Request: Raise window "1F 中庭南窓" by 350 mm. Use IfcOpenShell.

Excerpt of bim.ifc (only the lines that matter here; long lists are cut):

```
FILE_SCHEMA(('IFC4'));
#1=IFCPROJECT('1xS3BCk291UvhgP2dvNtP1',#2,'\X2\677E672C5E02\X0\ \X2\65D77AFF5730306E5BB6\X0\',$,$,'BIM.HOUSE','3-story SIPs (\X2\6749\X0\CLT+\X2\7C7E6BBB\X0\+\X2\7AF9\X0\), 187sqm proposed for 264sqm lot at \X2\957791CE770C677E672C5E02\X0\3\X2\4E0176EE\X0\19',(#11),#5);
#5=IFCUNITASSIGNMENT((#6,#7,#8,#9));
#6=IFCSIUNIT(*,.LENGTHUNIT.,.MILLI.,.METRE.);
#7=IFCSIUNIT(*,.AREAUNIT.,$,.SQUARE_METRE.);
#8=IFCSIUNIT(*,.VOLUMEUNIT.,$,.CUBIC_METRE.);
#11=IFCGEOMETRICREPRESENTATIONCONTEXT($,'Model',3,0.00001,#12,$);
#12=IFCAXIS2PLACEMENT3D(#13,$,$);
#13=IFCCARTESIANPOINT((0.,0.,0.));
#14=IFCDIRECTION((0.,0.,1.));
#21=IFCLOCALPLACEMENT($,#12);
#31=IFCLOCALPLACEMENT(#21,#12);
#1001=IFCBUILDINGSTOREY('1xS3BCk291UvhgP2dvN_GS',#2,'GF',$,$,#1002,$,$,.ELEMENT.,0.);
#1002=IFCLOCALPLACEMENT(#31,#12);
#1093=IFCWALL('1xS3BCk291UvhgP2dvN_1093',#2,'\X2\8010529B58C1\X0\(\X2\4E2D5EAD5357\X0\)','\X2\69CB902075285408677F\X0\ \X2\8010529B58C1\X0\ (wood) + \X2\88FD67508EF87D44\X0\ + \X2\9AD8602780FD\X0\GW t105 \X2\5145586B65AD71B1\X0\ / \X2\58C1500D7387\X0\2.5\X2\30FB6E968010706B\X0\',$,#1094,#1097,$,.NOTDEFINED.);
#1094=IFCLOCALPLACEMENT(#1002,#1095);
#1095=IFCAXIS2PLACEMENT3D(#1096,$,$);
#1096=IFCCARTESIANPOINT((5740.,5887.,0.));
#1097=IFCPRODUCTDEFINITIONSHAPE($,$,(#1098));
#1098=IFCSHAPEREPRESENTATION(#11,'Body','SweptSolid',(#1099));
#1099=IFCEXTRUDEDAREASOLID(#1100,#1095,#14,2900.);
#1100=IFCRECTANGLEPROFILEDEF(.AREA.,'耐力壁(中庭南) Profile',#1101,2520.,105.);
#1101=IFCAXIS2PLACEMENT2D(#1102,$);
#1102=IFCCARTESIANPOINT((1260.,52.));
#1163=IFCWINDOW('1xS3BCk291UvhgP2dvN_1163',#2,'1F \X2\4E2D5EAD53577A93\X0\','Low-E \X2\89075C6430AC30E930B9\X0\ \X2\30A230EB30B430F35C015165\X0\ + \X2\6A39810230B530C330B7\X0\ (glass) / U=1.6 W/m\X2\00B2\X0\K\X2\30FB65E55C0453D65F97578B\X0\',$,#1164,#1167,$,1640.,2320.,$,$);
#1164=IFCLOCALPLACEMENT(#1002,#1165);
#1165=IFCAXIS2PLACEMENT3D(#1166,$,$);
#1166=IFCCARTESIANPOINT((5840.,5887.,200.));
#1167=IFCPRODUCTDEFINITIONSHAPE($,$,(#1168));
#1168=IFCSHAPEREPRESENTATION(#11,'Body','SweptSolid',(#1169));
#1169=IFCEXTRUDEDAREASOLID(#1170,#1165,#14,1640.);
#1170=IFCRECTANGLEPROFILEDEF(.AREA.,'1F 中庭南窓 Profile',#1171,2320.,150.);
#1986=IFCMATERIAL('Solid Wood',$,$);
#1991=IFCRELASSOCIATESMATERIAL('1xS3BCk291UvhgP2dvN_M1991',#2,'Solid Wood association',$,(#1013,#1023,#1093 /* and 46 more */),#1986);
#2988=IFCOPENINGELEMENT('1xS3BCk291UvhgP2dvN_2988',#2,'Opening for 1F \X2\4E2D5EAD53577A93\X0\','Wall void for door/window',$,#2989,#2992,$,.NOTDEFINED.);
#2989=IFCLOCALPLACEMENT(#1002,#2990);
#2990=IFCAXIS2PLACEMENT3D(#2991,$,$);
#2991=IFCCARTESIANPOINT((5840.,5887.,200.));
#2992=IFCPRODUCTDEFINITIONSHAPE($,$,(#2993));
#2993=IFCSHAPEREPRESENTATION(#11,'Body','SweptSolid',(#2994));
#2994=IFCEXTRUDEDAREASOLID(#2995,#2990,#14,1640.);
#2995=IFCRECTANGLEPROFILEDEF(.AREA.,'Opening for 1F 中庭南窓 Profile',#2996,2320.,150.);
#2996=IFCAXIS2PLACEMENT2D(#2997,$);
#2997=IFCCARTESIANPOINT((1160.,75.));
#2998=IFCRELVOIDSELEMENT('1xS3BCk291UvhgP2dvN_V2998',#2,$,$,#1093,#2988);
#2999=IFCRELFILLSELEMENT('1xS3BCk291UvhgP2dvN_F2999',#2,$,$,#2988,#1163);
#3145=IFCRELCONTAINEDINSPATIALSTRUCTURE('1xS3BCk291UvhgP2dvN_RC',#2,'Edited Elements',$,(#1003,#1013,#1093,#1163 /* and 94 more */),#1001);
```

```python
import numpy as np
import ifcopenshell
import ifcopenshell.api.geometry
import ifcopenshell.util.placement
import ifcopenshell.util.unit

model = ifcopenshell.open("bim.ifc")
unit_scale = ifcopenshell.util.unit.calculate_unit_scale(model)

window = model.by_id(1163)
opening = window.FillsVoids[0].RelatingOpeningElement
dz = 0.35 / unit_scale

shift = np.array([0.0, 0.0, dz])
# The window is not placed relative to its opening, so move both.
for product in (opening, window):
    matrix = ifcopenshell.util.placement.get_local_placement(product.ObjectPlacement)
    matrix[:3, 3] += shift
    ifcopenshell.api.geometry.edit_object_placement(model, product=product, matrix=matrix, is_si=False)

print(f"moved by {dz * unit_scale:+.3f} m")

model.write("bim-out.ifc")
```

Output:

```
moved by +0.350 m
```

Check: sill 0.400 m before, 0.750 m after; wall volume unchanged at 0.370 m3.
